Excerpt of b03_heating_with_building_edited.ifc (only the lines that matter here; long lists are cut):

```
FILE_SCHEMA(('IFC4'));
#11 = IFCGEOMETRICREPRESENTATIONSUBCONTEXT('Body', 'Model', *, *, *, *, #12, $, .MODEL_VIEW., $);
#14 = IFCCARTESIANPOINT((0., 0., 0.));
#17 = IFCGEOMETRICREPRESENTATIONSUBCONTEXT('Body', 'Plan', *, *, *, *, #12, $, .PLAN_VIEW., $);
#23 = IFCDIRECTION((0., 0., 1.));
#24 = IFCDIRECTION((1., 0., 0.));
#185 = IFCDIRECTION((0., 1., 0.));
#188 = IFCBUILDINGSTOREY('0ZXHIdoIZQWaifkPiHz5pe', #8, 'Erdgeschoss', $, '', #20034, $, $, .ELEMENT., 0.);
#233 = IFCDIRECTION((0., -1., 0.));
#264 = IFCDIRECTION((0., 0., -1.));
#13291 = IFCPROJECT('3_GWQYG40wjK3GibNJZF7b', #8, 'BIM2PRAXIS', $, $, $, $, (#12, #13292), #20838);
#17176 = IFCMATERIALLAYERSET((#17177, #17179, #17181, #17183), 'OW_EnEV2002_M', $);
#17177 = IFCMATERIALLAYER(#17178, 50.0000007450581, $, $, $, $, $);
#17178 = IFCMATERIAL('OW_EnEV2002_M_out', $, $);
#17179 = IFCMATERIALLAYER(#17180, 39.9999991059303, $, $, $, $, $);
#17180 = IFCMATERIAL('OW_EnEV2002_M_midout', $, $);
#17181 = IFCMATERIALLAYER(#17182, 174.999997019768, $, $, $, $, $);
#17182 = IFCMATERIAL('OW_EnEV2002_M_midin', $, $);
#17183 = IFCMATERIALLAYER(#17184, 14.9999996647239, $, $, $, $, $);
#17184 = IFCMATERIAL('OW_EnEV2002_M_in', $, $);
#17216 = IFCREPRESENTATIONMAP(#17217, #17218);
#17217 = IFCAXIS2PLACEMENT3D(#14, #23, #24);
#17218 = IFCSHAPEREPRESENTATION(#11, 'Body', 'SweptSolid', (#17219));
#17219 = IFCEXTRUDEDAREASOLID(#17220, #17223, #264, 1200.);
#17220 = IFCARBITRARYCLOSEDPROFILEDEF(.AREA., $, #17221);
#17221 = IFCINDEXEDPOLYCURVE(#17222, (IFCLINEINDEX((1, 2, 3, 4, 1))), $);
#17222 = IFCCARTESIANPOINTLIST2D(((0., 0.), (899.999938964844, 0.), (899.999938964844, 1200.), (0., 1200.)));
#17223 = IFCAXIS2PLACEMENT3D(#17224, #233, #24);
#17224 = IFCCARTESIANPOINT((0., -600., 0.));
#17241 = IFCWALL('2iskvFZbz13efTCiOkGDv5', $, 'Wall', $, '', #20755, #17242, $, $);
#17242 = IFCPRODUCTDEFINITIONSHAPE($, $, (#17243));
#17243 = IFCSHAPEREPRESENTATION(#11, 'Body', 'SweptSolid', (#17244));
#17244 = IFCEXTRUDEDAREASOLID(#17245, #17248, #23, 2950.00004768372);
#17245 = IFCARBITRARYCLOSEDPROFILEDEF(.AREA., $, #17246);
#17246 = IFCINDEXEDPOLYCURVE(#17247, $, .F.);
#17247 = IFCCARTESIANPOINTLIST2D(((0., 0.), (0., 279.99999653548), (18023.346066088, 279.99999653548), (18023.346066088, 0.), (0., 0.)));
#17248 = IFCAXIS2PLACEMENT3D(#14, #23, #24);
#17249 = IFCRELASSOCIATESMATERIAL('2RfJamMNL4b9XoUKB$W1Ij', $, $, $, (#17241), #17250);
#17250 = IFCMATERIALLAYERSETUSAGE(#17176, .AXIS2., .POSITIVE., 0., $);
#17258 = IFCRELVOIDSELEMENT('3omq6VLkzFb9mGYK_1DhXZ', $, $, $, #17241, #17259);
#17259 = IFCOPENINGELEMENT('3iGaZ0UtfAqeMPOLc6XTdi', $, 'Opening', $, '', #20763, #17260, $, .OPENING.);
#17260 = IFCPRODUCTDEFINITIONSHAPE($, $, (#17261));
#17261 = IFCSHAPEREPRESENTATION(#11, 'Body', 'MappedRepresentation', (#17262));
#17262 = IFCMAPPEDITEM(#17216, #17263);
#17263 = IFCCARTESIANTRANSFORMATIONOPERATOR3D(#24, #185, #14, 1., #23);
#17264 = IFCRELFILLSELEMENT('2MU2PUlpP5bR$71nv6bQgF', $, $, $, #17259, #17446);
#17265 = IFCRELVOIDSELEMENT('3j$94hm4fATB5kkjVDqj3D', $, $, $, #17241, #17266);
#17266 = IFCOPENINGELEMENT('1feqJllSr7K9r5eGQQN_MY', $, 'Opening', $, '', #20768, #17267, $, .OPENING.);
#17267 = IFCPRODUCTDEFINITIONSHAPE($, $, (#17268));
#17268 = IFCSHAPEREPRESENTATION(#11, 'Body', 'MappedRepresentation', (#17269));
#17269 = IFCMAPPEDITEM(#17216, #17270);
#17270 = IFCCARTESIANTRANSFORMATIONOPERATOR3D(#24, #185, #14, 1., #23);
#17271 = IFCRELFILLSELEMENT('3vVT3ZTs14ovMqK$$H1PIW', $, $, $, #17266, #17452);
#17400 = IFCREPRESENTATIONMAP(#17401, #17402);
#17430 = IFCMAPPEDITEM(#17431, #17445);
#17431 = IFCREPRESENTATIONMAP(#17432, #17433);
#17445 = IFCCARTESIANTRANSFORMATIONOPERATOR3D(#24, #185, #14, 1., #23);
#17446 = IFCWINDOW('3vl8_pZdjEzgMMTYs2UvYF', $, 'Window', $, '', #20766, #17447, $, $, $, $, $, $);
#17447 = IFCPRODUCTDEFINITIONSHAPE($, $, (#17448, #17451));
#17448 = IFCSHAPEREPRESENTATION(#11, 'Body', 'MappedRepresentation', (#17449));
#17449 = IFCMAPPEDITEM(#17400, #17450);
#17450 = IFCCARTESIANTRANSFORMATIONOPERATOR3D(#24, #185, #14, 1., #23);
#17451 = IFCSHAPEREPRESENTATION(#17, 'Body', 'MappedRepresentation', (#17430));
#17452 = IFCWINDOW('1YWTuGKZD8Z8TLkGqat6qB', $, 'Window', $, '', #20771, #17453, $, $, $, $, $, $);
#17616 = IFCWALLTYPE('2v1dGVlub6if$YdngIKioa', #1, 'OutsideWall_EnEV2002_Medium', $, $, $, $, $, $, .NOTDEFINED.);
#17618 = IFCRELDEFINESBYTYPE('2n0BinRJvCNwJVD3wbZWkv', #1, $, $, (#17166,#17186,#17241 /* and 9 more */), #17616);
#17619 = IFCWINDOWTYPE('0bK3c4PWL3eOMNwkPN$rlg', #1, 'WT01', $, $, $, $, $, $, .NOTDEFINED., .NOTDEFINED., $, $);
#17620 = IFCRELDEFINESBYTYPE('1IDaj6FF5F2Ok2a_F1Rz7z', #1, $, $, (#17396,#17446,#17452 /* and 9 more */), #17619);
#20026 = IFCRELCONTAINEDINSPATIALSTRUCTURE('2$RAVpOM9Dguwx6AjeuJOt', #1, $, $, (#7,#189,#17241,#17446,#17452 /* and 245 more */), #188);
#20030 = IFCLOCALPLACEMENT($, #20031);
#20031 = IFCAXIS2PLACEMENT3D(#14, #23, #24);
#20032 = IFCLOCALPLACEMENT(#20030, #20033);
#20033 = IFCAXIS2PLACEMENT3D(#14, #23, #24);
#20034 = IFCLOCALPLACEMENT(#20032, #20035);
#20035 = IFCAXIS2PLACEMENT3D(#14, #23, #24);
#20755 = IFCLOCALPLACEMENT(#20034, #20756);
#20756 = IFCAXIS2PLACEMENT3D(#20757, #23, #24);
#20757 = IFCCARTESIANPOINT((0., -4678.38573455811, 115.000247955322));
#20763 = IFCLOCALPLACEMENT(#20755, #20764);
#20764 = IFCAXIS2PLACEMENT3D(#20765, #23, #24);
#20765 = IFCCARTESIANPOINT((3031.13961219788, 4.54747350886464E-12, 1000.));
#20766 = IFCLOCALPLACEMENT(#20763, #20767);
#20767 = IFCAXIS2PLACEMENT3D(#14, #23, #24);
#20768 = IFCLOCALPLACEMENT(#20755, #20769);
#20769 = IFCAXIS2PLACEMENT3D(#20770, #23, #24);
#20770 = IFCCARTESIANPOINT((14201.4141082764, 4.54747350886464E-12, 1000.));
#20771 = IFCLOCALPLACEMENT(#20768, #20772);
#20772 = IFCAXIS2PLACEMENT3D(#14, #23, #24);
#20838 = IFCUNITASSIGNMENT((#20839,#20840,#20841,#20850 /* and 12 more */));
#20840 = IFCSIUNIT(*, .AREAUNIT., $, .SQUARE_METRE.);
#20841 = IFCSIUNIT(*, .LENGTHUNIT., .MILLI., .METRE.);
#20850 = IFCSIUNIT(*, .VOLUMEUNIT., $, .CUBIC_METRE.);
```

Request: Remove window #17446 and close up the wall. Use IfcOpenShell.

```python
import ifcopenshell
import ifcopenshell.api.feature
import ifcopenshell.api.root
import ifcopenshell.geom
import ifcopenshell.util.shape

model = ifcopenshell.open("b03_heating_with_building_edited.ifc")
settings = ifcopenshell.geom.settings()


def volume(element):
    """Net volume in cubic metres, openings subtracted."""
    shape = ifcopenshell.geom.create_shape(settings, element)
    return ifcopenshell.util.shape.get_volume(shape.geometry)


window = model.by_guid("3vl8_pZdjEzgMMTYs2UvYF")
opening = window.FillsVoids[0].RelatingOpeningElement
wall = opening.VoidsElements[0].RelatingBuildingElement
before = volume(wall)

ifcopenshell.api.root.remove_product(model, product=window)
ifcopenshell.api.feature.remove_feature(model, feature=opening)

after = volume(wall)

print(f"wall volume {before:.3f} -> {after:.3f} m3")

model.write("b03_heating_with_building_edited_v2.ifc")
```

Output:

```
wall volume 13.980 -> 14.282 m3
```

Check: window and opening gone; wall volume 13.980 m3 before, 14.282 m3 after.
